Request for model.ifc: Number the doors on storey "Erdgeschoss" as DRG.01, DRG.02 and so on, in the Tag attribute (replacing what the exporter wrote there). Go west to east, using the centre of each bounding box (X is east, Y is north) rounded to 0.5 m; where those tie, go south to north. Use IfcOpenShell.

First a look at what the model holds.

```python
import ifcopenshell
import ifcopenshell.util.element
import ifcopenshell.util.placement

model = ifcopenshell.open("model.ifc")
print(model.schema)
storey = next(s for s in model.by_type("IfcBuildingStorey") if s.Name == "Erdgeschoss")
doors = [e for e in ifcopenshell.util.element.get_decomposition(storey) if e.is_a("IfcDoor")]
for e in sorted(doors, key=lambda e: e.id()):
    origin = ifcopenshell.util.placement.get_local_placement(e.ObjectPlacement)[:3, 3]
    print(e.id(), e.Tag, e.Name, origin.round(2) + 0.0, sep=" | ")
```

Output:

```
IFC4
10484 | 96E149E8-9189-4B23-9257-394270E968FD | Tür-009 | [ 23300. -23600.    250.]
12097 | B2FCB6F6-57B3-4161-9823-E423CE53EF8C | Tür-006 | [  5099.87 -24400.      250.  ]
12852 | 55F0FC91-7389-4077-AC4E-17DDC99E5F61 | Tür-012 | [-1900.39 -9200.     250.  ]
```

```python
import ifcopenshell
import ifcopenshell.geom
import ifcopenshell.util.element
import ifcopenshell.util.shape

model = ifcopenshell.open("model.ifc")
settings = ifcopenshell.geom.settings()
settings.set("use-world-coords", True)


def centre(element):
    shape = ifcopenshell.geom.create_shape(settings, element)
    return ifcopenshell.util.shape.get_bbox_centroid(shape.geometry)


storey = next(s for s in model.by_type("IfcBuildingStorey") if s.Name == "Erdgeschoss")
doors = [e for e in ifcopenshell.util.element.get_decomposition(storey) if e.is_a("IfcDoor")]

# Insertion points can sit at a corner or the storey origin, so sort by the geometry (in metres).
centres = {e: centre(e) for e in doors}
doors.sort(key=lambda e: (round(centres[e][0] / 0.5), centres[e][1]))

for i, e in enumerate(doors, start=1):
    number = f"DRG.{i:02d}"
    e.Tag = number
    print(e.id(), number)

model.write("model_rev.ifc")
```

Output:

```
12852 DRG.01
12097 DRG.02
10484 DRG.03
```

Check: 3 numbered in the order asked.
